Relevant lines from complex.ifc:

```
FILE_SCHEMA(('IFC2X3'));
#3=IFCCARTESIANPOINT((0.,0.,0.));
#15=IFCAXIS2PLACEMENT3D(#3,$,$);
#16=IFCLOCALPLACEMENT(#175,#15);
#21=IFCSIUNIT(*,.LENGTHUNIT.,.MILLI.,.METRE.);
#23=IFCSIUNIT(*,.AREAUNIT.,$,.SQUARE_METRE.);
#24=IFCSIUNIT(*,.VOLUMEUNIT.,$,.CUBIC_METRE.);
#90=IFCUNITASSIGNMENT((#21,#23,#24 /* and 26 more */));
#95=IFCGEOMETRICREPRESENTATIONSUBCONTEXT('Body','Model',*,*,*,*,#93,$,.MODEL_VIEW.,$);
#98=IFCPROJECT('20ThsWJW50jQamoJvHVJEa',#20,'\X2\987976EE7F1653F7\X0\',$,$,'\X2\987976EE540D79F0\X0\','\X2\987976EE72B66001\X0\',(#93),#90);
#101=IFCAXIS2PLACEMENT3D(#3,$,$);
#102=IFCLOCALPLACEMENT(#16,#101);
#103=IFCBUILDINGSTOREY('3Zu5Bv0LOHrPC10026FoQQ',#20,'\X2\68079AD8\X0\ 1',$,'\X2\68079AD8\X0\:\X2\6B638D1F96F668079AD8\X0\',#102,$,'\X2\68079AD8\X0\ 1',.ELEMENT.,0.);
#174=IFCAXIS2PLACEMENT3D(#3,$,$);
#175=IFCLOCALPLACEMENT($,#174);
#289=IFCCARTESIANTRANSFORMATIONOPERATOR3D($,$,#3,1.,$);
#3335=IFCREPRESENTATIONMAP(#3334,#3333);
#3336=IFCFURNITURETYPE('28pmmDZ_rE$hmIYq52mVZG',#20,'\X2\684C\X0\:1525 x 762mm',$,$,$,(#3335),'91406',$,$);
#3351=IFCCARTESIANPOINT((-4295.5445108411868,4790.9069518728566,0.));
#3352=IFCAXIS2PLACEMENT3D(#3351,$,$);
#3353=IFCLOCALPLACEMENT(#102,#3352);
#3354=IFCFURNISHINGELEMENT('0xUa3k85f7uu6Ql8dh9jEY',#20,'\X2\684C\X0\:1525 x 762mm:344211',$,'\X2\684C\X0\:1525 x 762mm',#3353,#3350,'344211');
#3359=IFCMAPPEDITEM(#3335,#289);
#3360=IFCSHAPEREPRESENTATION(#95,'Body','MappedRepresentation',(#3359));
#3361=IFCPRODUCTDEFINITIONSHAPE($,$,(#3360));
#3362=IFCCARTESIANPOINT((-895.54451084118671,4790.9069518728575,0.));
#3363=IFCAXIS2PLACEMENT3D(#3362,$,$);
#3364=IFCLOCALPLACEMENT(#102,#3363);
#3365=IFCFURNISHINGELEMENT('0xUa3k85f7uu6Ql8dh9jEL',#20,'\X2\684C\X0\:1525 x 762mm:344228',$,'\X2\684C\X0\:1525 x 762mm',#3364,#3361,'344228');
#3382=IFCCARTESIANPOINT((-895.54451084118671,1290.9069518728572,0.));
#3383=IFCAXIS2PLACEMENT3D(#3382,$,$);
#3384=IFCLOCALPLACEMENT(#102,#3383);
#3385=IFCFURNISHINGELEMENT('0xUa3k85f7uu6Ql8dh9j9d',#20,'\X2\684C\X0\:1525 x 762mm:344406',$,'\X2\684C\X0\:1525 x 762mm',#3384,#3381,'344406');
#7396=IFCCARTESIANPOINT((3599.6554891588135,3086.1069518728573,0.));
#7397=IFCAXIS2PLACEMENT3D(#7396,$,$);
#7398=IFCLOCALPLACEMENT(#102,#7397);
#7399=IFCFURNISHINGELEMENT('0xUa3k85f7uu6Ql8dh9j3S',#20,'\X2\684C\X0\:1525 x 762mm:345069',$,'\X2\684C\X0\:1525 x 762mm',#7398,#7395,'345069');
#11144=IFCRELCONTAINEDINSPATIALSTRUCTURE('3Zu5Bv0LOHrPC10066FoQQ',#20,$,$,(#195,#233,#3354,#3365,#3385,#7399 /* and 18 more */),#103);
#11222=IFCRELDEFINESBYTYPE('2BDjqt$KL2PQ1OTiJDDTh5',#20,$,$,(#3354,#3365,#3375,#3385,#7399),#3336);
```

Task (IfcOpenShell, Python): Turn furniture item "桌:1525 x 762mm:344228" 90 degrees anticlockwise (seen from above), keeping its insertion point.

```python
import ifcopenshell
import ifcopenshell.api.geometry
import ifcopenshell.util.placement

model = ifcopenshell.open("complex.ifc")

item = model.by_guid("0xUa3k85f7uu6Ql8dh9jEL")
matrix = ifcopenshell.util.placement.get_local_placement(item.ObjectPlacement)
matrix = matrix @ ifcopenshell.util.placement.rotation(90, "Z")
ifcopenshell.api.geometry.edit_object_placement(model, product=item, matrix=matrix, is_si=False)

print(ifcopenshell.util.placement.get_local_placement(item.ObjectPlacement).round(3) + 0.0)

model.write("complex_edited.ifc")
```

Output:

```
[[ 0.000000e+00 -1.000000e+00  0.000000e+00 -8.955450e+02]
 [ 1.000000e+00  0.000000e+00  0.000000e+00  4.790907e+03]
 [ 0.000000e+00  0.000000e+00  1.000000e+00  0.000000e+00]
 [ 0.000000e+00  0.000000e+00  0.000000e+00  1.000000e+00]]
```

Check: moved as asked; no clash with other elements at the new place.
